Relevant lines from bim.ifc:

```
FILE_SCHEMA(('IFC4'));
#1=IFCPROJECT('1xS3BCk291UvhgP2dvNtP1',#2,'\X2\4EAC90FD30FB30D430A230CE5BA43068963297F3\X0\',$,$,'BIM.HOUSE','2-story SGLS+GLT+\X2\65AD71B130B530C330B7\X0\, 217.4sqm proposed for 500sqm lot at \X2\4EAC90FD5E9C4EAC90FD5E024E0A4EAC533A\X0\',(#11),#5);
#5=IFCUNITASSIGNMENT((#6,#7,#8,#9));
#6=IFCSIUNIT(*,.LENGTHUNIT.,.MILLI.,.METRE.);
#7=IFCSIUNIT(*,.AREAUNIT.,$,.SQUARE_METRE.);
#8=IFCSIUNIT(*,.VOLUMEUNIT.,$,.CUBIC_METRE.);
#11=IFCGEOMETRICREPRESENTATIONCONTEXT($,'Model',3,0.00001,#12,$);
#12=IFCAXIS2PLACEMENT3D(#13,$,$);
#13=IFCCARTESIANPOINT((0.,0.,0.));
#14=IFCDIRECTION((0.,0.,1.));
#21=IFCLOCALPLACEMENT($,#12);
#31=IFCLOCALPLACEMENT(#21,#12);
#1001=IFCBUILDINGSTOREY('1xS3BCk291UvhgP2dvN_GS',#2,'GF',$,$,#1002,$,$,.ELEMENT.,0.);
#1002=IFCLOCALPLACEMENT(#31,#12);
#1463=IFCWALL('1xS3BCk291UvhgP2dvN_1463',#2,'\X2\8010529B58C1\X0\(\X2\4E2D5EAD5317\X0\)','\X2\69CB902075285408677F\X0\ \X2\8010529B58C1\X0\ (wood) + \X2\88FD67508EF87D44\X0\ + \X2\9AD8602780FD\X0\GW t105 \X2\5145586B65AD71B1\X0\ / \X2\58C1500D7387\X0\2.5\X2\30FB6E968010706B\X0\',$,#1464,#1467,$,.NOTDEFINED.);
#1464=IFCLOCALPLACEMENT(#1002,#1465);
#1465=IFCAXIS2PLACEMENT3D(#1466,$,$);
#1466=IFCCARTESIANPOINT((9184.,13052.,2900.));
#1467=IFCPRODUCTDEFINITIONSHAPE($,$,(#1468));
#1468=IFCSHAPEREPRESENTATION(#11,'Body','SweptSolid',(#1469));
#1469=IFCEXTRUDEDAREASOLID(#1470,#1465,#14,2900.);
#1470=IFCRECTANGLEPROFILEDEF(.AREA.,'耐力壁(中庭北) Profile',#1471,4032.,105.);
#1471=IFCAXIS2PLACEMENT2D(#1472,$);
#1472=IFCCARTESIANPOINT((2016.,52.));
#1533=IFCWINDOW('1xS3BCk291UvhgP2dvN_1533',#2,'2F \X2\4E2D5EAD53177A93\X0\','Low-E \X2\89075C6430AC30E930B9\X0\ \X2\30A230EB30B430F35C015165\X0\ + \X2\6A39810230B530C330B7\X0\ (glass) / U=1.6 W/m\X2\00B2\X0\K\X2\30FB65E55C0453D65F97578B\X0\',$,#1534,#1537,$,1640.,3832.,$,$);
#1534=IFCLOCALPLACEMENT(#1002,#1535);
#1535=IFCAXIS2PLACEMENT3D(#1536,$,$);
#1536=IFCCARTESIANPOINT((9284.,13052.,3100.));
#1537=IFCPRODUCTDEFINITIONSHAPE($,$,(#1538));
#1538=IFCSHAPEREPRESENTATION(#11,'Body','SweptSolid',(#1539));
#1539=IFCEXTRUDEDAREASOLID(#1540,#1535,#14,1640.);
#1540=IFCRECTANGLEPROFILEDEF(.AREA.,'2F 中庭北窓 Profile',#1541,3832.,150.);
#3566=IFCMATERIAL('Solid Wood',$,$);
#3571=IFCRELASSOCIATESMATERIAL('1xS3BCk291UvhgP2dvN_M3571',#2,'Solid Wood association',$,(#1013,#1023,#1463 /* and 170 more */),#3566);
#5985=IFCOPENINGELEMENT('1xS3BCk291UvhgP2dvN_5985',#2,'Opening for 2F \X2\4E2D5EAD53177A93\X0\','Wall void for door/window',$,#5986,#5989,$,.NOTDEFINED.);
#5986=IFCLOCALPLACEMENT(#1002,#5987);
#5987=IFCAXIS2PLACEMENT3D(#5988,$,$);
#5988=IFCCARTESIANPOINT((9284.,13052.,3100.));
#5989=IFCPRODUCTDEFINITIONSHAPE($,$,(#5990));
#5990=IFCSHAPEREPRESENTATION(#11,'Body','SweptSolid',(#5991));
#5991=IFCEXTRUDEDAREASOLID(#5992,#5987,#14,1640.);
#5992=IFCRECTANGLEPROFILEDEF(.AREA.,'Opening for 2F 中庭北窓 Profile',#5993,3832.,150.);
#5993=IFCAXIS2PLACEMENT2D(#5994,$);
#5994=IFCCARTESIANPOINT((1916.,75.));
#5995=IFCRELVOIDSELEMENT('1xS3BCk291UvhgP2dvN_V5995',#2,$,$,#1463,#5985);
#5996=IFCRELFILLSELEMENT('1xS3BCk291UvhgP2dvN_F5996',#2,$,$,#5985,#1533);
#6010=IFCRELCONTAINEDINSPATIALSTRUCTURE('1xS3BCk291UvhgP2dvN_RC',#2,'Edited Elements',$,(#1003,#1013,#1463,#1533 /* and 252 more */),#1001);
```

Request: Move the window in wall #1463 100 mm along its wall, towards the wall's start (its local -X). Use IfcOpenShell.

```python
import ifcopenshell
import ifcopenshell.api.geometry
import ifcopenshell.util.placement
import ifcopenshell.util.unit

model = ifcopenshell.open("bim.ifc")
unit_scale = ifcopenshell.util.unit.calculate_unit_scale(model)

window = model.by_id(1533)
opening = window.FillsVoids[0].RelatingOpeningElement
wall = opening.VoidsElements[0].RelatingBuildingElement

wall_matrix = ifcopenshell.util.placement.get_local_placement(wall.ObjectPlacement)
shift = wall_matrix[:3, 0] * -0.1 / unit_scale
before = ifcopenshell.util.placement.get_local_placement(window.ObjectPlacement)[:3, 3].copy()

# The window is not placed relative to its opening, so move both.
for product in (opening, window):
    matrix = ifcopenshell.util.placement.get_local_placement(product.ObjectPlacement)
    matrix[:3, 3] += shift
    ifcopenshell.api.geometry.edit_object_placement(model, product=product, matrix=matrix, is_si=False)

after = ifcopenshell.util.placement.get_local_placement(window.ObjectPlacement)[:3, 3]
print("window moved by", (after - before).round(3) + 0.0)

model.write("bim_edited.ifc")
```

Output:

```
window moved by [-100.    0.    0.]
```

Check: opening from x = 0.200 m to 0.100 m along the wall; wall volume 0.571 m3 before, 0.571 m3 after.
